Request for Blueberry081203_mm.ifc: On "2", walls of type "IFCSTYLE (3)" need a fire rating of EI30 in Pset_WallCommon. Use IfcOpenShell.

First a look at what the model holds.

```python
import ifcopenshell
import ifcopenshell.util.element

model = ifcopenshell.open("Blueberry081203_mm.ifc")
print(model.schema)
storey = next(s for s in model.by_type("IfcBuildingStorey") if s.Name == "2")
walls = [e for e in ifcopenshell.util.element.get_decomposition(storey) if e.is_a("IfcWall")]
seen = {}
for e in walls:
    element_type = ifcopenshell.util.element.get_type(e)
    key = (element_type.Name if element_type != e and element_type else None, ifcopenshell.util.element.get_pset(e, "Pset_WallCommon", "FireRating"))
    seen[key] = seen.get(key, 0) + 1
for (name, value), count in sorted(seen.items(), key=str):
    print(count, "x", name, "|", value)
```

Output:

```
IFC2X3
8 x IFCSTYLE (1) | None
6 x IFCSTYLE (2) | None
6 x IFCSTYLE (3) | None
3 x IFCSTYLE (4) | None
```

```python
import ifcopenshell
import ifcopenshell.api.pset
import ifcopenshell.util.element

model = ifcopenshell.open("Blueberry081203_mm.ifc")

storey = next(s for s in model.by_type("IfcBuildingStorey") if s.Name == "2")
walls = [e for e in ifcopenshell.util.element.get_decomposition(storey) if e.is_a("IfcWall")]

count = 0
for e in walls:
    element_type = ifcopenshell.util.element.get_type(e)
    if element_type in (None, e) or element_type.Name != "IFCSTYLE (3)":
        continue
    # add_pset returns the element's existing set when there is one.
    pset = ifcopenshell.api.pset.add_pset(model, product=e, name="Pset_WallCommon")
    ifcopenshell.api.pset.edit_pset(model, pset=pset, properties={"FireRating": "EI30"})
    count += 1

print(count, "walls updated")

model.write("Blueberry081203_mm_updated.ifc")
```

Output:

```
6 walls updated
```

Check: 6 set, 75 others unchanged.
